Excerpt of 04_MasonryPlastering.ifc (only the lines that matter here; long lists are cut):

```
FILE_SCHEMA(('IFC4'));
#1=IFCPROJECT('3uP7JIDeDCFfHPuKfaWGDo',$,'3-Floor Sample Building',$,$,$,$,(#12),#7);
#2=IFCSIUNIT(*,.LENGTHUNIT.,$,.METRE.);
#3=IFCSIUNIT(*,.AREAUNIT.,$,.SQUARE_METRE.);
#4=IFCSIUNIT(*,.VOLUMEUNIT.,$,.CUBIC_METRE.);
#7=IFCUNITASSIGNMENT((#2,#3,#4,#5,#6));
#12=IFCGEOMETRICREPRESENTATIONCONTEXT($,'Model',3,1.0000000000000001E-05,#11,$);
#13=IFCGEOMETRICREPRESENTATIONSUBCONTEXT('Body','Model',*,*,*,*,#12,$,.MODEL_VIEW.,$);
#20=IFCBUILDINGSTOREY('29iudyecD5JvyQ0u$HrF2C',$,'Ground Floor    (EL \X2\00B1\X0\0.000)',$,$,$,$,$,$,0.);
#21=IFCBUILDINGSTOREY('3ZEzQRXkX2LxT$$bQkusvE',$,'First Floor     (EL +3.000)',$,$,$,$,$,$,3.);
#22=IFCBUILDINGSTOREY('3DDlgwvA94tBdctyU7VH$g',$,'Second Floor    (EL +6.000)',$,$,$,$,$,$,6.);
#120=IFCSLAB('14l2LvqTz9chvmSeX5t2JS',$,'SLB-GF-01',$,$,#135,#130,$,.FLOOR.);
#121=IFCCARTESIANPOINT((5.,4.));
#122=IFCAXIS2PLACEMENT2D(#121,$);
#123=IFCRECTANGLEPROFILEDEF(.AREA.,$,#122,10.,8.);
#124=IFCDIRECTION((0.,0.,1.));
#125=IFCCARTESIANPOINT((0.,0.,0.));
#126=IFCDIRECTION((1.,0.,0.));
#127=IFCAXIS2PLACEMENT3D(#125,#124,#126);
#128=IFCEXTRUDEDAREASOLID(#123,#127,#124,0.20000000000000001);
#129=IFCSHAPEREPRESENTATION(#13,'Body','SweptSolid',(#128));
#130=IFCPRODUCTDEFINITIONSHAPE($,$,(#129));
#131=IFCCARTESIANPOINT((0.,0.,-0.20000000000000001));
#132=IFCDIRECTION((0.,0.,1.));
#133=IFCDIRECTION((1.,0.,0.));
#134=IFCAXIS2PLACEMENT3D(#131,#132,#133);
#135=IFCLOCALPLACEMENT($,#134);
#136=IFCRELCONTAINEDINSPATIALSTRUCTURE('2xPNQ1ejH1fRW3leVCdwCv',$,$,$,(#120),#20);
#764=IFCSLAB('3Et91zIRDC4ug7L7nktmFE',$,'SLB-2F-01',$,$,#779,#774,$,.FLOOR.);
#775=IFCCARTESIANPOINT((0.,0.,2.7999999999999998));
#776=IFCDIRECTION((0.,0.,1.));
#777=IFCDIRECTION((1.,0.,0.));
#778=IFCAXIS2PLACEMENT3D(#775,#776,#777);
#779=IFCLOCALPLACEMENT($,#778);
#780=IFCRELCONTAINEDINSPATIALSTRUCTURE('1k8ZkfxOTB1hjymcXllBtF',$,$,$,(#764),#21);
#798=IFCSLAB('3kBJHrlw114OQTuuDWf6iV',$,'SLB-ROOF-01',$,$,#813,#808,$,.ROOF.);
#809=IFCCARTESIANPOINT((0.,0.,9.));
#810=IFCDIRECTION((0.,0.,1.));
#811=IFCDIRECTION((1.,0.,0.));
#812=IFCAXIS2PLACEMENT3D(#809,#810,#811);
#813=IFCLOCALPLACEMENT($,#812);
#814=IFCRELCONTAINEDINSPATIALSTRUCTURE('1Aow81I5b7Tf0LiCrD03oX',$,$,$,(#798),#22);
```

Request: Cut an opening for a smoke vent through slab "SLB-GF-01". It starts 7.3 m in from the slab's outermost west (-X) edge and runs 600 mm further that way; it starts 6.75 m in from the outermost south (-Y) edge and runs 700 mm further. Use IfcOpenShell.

```python
import numpy as np
import ifcopenshell
import ifcopenshell.api.feature
import ifcopenshell.api.geometry
import ifcopenshell.api.root
import ifcopenshell.geom
import ifcopenshell.util.placement
import ifcopenshell.util.representation
import ifcopenshell.util.shape
import ifcopenshell.util.unit

model = ifcopenshell.open("04_MasonryPlastering.ifc")
unit_scale = ifcopenshell.util.unit.calculate_unit_scale(model)
settings = ifcopenshell.geom.settings()


def volume(element):
    """Net volume in cubic metres, openings subtracted."""
    shape = ifcopenshell.geom.create_shape(settings, element)
    return ifcopenshell.util.shape.get_volume(shape.geometry)


slab = model.by_guid("14l2LvqTz9chvmSeX5t2JS")
before = volume(slab)

# Extent in the slab's own axes, in metres. The edges named are its -X and -Y sides.
slab_shape = ifcopenshell.geom.create_shape(settings, slab)
vertices = ifcopenshell.util.shape.get_vertices(slab_shape.geometry)
x_min, y_min, bottom = vertices.min(axis=0)
top = vertices[:, 2].max()

opening = ifcopenshell.api.root.create_entity(model, ifc_class="IfcOpeningElement", name="Smoke vent opening", predefined_type="OPENING")
context = ifcopenshell.util.representation.get_context(model, "Model", "Body", "MODEL_VIEW")
width, depth = 0.6, 0.7
outline = [(0.0, 0.0), (width, 0.0), (width, depth), (0.0, depth), (0.0, 0.0)]
# Overshoot both faces by 50 mm so the cut is clean.
shape = ifcopenshell.api.geometry.add_slab_representation(
    model, context=context, depth=top - bottom + 0.1, polyline=outline
)
ifcopenshell.api.geometry.assign_representation(model, product=opening, representation=shape)

matrix = ifcopenshell.util.placement.get_local_placement(slab.ObjectPlacement)
matrix[:, 3] = matrix @ np.append(np.array([x_min + 7.3, y_min + 6.75, bottom - 0.05]) / unit_scale, 1.0)
ifcopenshell.api.geometry.edit_object_placement(model, product=opening, matrix=matrix, is_si=False)
ifcopenshell.api.feature.add_feature(model, feature=opening, element=slab)

after = volume(slab)

print(f"slab volume {before:.3f} -> {after:.3f} m3")

model.write("04_MasonryPlastering_updated.ifc")
```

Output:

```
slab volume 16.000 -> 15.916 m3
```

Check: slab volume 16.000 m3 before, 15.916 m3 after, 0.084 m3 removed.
